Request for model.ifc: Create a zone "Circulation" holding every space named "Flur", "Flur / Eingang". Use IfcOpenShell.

First a look at what the model holds.

```python
import ifcopenshell

model = ifcopenshell.open("model.ifc")
print(model.schema)
seen = {}
for space in model.by_type("IfcSpace"):
    seen[space.LongName] = seen.get(space.LongName, 0) + 1
for name, count in sorted(seen.items(), key=str):
    print(count, "x", name)
print("zones:", [z.Name for z in model.by_type("IfcZone")][:20])
```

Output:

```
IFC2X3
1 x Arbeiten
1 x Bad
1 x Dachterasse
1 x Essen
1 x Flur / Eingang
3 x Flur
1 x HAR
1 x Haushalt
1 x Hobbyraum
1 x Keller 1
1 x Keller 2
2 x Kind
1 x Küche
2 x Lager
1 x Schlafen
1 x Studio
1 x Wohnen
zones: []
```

```python
import ifcopenshell
import ifcopenshell.api.group
import ifcopenshell.api.root

model = ifcopenshell.open("model.ifc")

names = {"Flur", "Flur / Eingang"}
spaces = [s for s in model.by_type("IfcSpace") if s.LongName in names]

zone = ifcopenshell.api.root.create_entity(model, ifc_class="IfcZone", name="Circulation")
ifcopenshell.api.group.assign_group(model, products=spaces, group=zone)
print(len(spaces), "spaces in", zone.Name)

model.write("model_updated.ifc")
```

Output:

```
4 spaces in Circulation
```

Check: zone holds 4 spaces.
